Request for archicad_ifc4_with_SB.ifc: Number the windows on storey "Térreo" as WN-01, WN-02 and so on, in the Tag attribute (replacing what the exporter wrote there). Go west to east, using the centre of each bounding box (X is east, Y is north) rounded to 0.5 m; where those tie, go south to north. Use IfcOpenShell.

First a look at what the model holds.

```python
import ifcopenshell
import ifcopenshell.util.element
import ifcopenshell.util.placement

model = ifcopenshell.open("archicad_ifc4_with_SB.ifc")
print(model.schema)
storey = next(s for s in model.by_type("IfcBuildingStorey") if s.Name == "Térreo")
windows = [e for e in ifcopenshell.util.element.get_decomposition(storey) if e.is_a("IfcWindow")]
for e in sorted(windows, key=lambda e: e.id()):
    origin = ifcopenshell.util.placement.get_local_placement(e.ObjectPlacement)[:3, 3]
    print(e.id(), e.Tag, e.Name, origin.round(2) + 0.0, sep=" | ")
```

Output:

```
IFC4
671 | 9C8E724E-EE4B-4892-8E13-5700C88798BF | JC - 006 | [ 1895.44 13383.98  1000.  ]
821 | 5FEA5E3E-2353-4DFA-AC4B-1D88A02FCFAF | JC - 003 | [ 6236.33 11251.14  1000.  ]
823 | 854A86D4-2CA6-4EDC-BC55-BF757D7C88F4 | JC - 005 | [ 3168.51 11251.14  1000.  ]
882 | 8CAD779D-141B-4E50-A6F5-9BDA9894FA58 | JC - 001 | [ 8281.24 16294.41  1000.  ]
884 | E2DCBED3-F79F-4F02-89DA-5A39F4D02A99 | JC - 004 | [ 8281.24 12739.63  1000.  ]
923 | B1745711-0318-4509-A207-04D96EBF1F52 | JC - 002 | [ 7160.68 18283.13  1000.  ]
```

```python
import ifcopenshell
import ifcopenshell.geom
import ifcopenshell.util.element
import ifcopenshell.util.shape

model = ifcopenshell.open("archicad_ifc4_with_SB.ifc")
settings = ifcopenshell.geom.settings()
settings.set("use-world-coords", True)


def centre(element):
    shape = ifcopenshell.geom.create_shape(settings, element)
    return ifcopenshell.util.shape.get_bbox_centroid(shape.geometry)


storey = next(s for s in model.by_type("IfcBuildingStorey") if s.Name == "Térreo")
windows = [e for e in ifcopenshell.util.element.get_decomposition(storey) if e.is_a("IfcWindow")]

# Insertion points can sit at a corner or the storey origin, so sort by the geometry (in metres).
centres = {e: centre(e) for e in windows}
windows.sort(key=lambda e: (round(centres[e][0] / 0.5), centres[e][1]))

for i, e in enumerate(windows, start=1):
    number = f"WN-{i:02d}"
    e.Tag = number
    print(e.id(), number)

model.write("archicad_ifc4_with_SB-out.ifc")
```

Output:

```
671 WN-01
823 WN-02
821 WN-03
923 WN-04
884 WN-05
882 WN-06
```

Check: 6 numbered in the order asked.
